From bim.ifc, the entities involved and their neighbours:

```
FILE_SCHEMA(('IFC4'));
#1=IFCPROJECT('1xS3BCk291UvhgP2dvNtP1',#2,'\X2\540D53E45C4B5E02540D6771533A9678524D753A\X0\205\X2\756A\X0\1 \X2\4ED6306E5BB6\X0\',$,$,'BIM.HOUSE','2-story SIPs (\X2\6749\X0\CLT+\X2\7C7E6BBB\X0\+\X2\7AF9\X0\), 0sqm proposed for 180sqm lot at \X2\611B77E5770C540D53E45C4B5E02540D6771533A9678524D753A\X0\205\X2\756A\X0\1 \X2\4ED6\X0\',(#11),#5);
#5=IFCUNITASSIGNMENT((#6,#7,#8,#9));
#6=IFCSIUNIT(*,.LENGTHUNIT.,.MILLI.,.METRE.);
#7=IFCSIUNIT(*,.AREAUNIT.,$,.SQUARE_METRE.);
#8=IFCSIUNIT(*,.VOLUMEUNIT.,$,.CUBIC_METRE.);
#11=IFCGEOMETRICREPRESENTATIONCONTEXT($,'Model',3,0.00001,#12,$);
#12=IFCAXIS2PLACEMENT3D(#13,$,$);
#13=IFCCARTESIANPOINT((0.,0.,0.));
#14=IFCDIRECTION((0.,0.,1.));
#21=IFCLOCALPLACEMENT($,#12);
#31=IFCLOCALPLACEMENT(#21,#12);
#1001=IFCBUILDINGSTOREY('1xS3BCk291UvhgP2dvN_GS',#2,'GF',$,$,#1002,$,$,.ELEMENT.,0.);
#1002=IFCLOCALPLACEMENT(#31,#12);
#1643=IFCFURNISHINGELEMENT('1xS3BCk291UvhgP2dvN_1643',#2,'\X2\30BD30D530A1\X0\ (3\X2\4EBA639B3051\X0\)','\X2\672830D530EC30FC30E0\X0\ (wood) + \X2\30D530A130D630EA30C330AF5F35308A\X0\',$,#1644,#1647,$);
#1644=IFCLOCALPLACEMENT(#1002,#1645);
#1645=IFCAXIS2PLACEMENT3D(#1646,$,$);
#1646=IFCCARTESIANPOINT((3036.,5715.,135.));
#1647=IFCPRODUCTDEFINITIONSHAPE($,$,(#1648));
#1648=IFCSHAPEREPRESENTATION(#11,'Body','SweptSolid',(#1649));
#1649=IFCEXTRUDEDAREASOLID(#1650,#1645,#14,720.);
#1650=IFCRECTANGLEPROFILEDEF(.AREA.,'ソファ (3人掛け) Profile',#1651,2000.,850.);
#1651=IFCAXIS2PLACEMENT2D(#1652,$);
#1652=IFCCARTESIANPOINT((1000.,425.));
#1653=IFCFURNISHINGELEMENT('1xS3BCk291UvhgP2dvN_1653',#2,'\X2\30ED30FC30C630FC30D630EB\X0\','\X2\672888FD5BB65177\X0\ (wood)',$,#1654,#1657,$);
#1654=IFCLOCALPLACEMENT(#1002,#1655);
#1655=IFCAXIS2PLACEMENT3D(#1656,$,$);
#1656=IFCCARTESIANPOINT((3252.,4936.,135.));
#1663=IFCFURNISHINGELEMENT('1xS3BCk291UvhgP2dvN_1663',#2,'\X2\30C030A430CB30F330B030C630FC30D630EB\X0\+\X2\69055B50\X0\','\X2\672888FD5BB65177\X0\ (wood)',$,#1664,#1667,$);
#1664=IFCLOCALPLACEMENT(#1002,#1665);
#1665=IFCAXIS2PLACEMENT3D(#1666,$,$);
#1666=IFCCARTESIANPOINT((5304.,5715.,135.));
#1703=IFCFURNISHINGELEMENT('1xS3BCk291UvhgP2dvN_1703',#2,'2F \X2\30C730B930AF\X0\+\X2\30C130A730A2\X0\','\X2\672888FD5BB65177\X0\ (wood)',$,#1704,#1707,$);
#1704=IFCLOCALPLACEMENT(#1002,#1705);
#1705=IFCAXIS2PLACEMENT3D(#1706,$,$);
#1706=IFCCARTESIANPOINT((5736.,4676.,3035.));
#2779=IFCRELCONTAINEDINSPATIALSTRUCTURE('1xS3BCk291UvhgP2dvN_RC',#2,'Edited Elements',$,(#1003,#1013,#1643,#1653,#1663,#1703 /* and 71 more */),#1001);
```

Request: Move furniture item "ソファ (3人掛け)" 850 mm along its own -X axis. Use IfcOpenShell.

```python
import ifcopenshell
import ifcopenshell.api.geometry
import ifcopenshell.util.placement
import ifcopenshell.util.unit

model = ifcopenshell.open("bim.ifc")
unit_scale = ifcopenshell.util.unit.calculate_unit_scale(model)

item = model.by_guid("1xS3BCk291UvhgP2dvN_1643")
matrix = ifcopenshell.util.placement.get_local_placement(item.ObjectPlacement)
matrix[:3, 3] -= matrix[:3, 0] * 0.85 / unit_scale
ifcopenshell.api.geometry.edit_object_placement(model, product=item, matrix=matrix, is_si=False)

print(ifcopenshell.util.placement.get_local_placement(item.ObjectPlacement).round(3) + 0.0)

model.write("bim_rev.ifc")
```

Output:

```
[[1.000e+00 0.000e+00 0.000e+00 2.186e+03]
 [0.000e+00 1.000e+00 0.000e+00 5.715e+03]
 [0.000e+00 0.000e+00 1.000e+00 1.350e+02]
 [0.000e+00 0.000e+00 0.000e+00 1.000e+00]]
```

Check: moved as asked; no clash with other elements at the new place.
